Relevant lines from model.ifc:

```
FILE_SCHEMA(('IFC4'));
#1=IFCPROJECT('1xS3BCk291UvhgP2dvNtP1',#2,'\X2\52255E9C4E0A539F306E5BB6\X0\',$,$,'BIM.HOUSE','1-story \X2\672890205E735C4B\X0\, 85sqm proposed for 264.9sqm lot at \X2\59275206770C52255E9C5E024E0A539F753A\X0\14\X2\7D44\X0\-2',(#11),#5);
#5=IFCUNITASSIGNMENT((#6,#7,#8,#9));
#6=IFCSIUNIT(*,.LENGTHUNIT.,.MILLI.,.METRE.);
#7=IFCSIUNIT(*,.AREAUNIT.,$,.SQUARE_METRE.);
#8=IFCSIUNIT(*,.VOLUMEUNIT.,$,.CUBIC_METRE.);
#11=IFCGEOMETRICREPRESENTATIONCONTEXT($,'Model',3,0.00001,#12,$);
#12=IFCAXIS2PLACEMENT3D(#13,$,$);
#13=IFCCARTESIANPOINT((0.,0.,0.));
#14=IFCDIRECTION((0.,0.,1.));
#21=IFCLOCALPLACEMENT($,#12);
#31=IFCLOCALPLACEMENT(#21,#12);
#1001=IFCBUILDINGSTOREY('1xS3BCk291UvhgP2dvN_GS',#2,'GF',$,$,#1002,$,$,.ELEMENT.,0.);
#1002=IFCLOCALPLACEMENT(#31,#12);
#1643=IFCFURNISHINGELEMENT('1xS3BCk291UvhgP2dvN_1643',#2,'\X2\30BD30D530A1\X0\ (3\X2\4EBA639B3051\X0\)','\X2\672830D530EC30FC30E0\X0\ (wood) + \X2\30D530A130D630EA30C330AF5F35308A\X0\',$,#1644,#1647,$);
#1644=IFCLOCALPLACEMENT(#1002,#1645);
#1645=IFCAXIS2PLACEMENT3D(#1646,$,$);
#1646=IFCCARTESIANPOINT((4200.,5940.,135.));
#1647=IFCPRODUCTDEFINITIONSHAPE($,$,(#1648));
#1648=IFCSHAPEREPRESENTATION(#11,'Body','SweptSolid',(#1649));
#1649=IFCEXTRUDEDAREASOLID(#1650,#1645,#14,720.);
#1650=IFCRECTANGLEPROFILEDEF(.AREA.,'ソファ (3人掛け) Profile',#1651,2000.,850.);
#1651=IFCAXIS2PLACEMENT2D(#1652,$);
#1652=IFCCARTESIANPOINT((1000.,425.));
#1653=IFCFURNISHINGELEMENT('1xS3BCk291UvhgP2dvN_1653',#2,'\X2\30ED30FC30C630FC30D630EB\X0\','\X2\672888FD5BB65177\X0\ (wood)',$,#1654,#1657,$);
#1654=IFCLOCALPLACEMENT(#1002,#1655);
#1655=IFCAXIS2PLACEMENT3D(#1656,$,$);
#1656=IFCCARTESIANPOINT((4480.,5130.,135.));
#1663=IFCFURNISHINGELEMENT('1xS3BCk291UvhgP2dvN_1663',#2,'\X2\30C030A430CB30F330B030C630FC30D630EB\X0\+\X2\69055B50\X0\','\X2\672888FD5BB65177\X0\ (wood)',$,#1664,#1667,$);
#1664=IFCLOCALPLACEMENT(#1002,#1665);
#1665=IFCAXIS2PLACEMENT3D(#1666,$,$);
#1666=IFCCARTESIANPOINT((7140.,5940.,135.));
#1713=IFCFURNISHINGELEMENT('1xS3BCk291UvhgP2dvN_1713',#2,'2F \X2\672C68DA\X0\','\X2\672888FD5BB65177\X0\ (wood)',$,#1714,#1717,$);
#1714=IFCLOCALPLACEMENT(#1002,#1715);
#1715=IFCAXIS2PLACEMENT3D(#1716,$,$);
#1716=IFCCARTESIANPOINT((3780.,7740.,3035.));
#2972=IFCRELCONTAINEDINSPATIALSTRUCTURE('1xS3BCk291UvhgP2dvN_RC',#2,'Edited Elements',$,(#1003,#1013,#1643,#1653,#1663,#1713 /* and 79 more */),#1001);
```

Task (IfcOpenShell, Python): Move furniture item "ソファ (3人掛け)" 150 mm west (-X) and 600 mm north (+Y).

```python
import ifcopenshell
import ifcopenshell.api.geometry
import ifcopenshell.util.placement

model = ifcopenshell.open("model.ifc")

item = model.by_guid("1xS3BCk291UvhgP2dvN_1643")
matrix = ifcopenshell.util.placement.get_local_placement(item.ObjectPlacement)
matrix[0, 3] -= 150.0
matrix[1, 3] += 600.0
ifcopenshell.api.geometry.edit_object_placement(model, product=item, matrix=matrix, is_si=False)

print(ifcopenshell.util.placement.get_local_placement(item.ObjectPlacement).round(3) + 0.0)

model.write("model_rev.ifc")
```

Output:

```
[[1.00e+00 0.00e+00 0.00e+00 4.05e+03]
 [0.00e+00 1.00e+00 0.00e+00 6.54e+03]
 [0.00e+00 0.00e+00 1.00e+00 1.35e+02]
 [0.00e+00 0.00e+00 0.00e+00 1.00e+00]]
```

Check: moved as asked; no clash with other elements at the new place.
